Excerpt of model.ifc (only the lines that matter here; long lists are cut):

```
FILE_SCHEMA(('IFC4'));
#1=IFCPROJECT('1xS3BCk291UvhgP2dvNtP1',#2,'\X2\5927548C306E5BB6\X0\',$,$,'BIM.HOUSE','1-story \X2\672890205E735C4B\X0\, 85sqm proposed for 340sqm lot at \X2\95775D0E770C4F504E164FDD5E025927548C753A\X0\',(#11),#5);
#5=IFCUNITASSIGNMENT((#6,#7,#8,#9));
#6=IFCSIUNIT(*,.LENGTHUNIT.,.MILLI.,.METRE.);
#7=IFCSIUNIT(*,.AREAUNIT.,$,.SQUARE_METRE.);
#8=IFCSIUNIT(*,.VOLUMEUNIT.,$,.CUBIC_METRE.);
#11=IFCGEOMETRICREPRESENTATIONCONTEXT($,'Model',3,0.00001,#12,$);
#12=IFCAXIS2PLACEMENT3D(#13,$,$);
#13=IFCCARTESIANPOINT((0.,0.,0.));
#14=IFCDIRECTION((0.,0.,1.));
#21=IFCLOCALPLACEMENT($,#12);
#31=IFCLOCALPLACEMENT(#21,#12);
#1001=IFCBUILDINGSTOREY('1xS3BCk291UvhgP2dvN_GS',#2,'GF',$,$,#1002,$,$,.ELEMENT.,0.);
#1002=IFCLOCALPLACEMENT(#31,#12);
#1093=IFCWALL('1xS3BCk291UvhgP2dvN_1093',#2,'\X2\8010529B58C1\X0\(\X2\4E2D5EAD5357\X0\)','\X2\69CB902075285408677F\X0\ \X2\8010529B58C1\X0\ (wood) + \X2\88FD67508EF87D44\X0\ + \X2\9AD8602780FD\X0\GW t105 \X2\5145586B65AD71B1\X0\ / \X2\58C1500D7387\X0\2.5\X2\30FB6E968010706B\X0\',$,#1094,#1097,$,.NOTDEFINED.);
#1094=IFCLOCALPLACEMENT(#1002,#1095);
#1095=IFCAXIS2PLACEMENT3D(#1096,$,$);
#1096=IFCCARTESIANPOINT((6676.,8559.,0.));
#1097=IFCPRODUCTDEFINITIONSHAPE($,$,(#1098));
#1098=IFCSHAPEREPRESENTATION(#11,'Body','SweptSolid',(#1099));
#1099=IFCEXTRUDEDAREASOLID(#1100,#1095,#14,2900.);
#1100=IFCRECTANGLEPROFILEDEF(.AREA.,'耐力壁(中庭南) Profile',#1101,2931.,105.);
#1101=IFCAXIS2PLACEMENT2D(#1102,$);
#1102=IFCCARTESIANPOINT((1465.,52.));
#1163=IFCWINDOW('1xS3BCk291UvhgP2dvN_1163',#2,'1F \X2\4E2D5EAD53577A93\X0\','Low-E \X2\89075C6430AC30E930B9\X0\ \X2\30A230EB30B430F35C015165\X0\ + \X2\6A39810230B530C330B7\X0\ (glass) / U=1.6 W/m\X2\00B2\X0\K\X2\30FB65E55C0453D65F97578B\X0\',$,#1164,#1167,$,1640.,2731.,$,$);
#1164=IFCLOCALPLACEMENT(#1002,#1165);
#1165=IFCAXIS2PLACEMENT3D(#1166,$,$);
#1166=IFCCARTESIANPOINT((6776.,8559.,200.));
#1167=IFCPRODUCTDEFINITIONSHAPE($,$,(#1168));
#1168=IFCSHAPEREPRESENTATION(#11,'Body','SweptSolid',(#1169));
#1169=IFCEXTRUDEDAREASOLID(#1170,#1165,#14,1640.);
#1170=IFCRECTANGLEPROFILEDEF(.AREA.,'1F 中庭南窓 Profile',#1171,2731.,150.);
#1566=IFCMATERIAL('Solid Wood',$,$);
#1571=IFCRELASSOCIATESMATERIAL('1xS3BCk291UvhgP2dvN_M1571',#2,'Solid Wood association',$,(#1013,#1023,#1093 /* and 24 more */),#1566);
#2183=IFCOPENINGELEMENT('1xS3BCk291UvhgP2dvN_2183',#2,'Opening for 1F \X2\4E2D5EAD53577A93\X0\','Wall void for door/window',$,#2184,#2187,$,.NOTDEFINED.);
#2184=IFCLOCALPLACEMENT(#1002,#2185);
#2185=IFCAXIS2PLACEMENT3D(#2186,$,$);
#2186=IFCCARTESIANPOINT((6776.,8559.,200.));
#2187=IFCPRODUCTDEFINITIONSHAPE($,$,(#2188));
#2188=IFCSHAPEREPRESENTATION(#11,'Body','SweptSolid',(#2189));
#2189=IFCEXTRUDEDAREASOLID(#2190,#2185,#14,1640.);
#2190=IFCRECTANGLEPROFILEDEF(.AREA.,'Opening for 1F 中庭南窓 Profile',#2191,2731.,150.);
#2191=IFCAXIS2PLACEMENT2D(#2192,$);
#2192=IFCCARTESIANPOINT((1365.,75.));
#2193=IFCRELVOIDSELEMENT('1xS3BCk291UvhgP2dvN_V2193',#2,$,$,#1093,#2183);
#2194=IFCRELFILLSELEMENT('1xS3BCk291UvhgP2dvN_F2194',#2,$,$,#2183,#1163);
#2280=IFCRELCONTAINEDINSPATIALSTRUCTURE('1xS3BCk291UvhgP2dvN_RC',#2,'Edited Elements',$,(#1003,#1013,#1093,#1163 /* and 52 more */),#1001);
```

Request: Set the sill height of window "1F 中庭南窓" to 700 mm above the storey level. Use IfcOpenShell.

```python
import numpy as np
import ifcopenshell
import ifcopenshell.api.geometry
import ifcopenshell.geom
import ifcopenshell.util.element
import ifcopenshell.util.placement
import ifcopenshell.util.shape
import ifcopenshell.util.unit

model = ifcopenshell.open("model.ifc")
unit_scale = ifcopenshell.util.unit.calculate_unit_scale(model)

window = model.by_guid("1xS3BCk291UvhgP2dvN_1163")
opening = window.FillsVoids[0].RelatingOpeningElement
storey = ifcopenshell.util.element.get_container(window, ifc_class="IfcBuildingStorey")
level = ifcopenshell.util.placement.get_local_placement(storey.ObjectPlacement)[2, 3]

# The opening's origin need not be at the sill, so measure its lowest point.
shape = ifcopenshell.geom.create_shape(ifcopenshell.geom.settings(), opening)
bottom = ifcopenshell.util.shape.get_shape_bottom_elevation(shape, shape.geometry) / unit_scale
dz = level + 0.7 / unit_scale - bottom

shift = np.array([0.0, 0.0, dz])
# The window is not placed relative to its opening, so move both.
for product in (opening, window):
    matrix = ifcopenshell.util.placement.get_local_placement(product.ObjectPlacement)
    matrix[:3, 3] += shift
    ifcopenshell.api.geometry.edit_object_placement(model, product=product, matrix=matrix, is_si=False)

print(f"moved by {dz * unit_scale:+.3f} m")

model.write("model_edited.ifc")
```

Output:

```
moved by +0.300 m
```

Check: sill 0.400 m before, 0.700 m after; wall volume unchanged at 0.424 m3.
